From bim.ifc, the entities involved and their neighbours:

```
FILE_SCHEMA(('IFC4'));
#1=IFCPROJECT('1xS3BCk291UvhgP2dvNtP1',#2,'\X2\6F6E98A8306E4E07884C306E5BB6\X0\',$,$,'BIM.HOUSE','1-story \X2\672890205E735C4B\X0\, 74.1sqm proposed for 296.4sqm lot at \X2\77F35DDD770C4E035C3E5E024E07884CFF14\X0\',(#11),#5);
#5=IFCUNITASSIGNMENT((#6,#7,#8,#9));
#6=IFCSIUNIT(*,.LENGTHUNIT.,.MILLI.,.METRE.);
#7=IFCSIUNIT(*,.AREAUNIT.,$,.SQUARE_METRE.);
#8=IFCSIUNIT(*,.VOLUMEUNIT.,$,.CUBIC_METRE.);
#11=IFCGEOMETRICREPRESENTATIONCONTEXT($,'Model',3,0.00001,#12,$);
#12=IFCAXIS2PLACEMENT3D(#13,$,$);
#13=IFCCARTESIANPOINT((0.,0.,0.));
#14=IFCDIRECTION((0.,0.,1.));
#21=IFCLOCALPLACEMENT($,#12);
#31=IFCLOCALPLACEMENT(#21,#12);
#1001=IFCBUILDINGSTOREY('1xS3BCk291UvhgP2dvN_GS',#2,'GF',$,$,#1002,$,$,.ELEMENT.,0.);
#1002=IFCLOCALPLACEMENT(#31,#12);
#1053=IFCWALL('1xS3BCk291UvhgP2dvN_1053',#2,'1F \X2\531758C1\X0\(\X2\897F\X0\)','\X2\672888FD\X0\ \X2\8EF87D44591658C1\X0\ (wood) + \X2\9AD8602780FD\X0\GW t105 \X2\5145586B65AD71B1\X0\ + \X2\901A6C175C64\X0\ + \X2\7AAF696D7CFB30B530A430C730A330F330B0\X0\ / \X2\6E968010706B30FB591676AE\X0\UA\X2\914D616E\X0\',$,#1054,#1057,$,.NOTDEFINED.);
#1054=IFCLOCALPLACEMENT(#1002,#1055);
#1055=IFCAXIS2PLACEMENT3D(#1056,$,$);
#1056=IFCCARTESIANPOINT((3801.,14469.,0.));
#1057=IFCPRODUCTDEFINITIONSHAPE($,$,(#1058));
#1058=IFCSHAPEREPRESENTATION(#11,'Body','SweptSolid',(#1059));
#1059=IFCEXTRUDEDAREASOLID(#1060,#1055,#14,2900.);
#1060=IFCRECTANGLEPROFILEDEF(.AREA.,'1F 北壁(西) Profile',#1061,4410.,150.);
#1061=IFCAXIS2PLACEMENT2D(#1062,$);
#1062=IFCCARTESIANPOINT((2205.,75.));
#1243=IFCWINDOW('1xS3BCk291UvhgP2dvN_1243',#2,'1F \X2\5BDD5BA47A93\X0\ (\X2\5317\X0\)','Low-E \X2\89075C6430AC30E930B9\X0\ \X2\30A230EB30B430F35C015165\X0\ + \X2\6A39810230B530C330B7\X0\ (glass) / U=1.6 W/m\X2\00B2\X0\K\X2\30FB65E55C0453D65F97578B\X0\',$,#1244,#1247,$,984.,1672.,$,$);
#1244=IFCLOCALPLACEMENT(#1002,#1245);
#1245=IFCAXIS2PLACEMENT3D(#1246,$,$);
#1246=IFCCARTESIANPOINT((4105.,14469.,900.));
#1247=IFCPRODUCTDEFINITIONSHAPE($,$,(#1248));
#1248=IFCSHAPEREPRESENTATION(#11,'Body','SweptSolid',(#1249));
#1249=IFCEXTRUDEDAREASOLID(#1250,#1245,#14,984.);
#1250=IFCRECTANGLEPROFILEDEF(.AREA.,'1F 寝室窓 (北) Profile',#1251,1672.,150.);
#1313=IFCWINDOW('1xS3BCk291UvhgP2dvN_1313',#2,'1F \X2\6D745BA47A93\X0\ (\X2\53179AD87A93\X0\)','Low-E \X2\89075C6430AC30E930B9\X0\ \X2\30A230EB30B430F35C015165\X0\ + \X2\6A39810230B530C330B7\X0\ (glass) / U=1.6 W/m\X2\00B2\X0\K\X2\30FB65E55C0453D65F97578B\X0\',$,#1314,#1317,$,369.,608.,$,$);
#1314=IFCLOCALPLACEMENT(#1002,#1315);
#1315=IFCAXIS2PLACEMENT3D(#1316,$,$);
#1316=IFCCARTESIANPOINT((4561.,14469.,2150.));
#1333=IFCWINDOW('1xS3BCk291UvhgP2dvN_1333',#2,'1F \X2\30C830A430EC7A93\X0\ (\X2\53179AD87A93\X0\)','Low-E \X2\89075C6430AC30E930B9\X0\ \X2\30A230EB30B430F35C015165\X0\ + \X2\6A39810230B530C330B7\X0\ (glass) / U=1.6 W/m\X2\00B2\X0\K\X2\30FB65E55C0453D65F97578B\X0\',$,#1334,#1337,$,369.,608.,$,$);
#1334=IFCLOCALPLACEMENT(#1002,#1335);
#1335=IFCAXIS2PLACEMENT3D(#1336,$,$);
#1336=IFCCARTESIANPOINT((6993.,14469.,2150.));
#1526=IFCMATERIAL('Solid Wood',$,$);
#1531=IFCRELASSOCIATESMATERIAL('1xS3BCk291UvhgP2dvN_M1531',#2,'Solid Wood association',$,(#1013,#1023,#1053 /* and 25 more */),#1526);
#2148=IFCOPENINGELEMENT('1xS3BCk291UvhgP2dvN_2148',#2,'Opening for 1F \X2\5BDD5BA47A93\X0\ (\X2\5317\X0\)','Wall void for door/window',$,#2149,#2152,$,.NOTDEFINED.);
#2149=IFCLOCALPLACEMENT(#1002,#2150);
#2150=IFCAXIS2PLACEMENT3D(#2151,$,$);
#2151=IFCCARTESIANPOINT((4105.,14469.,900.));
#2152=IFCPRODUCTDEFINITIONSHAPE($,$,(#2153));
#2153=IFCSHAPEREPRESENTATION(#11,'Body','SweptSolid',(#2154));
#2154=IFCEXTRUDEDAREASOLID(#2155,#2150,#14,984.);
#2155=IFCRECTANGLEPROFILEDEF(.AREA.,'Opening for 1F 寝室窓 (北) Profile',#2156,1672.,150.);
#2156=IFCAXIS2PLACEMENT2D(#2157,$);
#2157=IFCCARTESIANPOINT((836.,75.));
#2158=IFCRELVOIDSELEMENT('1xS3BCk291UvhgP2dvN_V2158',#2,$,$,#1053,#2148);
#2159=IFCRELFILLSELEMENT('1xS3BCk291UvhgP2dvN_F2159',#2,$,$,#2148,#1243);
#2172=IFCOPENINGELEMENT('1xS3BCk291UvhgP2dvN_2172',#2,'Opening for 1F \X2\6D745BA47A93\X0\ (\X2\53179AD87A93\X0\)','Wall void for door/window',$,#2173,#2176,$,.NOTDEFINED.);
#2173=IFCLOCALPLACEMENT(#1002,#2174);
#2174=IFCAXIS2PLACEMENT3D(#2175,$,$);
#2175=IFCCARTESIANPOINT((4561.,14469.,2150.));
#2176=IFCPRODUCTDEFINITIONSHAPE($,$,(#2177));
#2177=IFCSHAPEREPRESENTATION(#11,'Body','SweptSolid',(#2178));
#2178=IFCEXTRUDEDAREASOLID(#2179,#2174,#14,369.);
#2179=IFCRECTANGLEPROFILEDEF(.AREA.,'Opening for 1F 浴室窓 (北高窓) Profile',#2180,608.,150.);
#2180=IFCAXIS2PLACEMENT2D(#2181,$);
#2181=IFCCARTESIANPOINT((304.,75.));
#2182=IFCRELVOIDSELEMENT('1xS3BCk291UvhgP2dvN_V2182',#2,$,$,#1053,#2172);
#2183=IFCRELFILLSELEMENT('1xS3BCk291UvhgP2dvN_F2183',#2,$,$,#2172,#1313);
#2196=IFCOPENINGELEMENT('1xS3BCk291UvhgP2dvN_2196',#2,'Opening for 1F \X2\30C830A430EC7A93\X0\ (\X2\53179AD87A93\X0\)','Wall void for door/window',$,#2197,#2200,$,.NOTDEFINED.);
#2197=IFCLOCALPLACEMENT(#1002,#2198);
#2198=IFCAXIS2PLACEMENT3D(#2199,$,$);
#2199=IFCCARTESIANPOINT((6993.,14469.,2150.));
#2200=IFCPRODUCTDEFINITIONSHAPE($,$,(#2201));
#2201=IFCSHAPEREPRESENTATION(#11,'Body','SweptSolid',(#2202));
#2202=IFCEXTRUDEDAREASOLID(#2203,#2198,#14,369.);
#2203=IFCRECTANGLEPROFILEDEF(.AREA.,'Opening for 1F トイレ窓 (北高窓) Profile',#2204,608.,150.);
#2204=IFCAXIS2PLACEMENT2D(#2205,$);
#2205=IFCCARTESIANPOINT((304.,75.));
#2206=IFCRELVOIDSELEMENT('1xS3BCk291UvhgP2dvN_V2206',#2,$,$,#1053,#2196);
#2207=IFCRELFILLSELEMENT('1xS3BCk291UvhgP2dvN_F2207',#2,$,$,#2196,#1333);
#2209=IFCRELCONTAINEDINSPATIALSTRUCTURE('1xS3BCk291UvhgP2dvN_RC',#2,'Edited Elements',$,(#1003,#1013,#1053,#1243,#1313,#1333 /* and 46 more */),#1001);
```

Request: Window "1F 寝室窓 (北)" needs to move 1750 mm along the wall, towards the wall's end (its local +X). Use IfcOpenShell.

```python
import ifcopenshell
import ifcopenshell.api.geometry
import ifcopenshell.util.placement
import ifcopenshell.util.unit

model = ifcopenshell.open("bim.ifc")
unit_scale = ifcopenshell.util.unit.calculate_unit_scale(model)

window = model.by_id(1243)
opening = window.FillsVoids[0].RelatingOpeningElement
wall = opening.VoidsElements[0].RelatingBuildingElement

wall_matrix = ifcopenshell.util.placement.get_local_placement(wall.ObjectPlacement)
shift = wall_matrix[:3, 0] * 1.75 / unit_scale
before = ifcopenshell.util.placement.get_local_placement(window.ObjectPlacement)[:3, 3].copy()

# The window is not placed relative to its opening, so move both.
for product in (opening, window):
    matrix = ifcopenshell.util.placement.get_local_placement(product.ObjectPlacement)
    matrix[:3, 3] += shift
    ifcopenshell.api.geometry.edit_object_placement(model, product=product, matrix=matrix, is_si=False)

after = ifcopenshell.util.placement.get_local_placement(window.ObjectPlacement)[:3, 3]
print("window moved by", (after - before).round(3) + 0.0)

model.write("bim_v2.ifc")
```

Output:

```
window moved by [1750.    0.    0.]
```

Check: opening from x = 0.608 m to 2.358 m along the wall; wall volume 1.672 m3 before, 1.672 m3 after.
